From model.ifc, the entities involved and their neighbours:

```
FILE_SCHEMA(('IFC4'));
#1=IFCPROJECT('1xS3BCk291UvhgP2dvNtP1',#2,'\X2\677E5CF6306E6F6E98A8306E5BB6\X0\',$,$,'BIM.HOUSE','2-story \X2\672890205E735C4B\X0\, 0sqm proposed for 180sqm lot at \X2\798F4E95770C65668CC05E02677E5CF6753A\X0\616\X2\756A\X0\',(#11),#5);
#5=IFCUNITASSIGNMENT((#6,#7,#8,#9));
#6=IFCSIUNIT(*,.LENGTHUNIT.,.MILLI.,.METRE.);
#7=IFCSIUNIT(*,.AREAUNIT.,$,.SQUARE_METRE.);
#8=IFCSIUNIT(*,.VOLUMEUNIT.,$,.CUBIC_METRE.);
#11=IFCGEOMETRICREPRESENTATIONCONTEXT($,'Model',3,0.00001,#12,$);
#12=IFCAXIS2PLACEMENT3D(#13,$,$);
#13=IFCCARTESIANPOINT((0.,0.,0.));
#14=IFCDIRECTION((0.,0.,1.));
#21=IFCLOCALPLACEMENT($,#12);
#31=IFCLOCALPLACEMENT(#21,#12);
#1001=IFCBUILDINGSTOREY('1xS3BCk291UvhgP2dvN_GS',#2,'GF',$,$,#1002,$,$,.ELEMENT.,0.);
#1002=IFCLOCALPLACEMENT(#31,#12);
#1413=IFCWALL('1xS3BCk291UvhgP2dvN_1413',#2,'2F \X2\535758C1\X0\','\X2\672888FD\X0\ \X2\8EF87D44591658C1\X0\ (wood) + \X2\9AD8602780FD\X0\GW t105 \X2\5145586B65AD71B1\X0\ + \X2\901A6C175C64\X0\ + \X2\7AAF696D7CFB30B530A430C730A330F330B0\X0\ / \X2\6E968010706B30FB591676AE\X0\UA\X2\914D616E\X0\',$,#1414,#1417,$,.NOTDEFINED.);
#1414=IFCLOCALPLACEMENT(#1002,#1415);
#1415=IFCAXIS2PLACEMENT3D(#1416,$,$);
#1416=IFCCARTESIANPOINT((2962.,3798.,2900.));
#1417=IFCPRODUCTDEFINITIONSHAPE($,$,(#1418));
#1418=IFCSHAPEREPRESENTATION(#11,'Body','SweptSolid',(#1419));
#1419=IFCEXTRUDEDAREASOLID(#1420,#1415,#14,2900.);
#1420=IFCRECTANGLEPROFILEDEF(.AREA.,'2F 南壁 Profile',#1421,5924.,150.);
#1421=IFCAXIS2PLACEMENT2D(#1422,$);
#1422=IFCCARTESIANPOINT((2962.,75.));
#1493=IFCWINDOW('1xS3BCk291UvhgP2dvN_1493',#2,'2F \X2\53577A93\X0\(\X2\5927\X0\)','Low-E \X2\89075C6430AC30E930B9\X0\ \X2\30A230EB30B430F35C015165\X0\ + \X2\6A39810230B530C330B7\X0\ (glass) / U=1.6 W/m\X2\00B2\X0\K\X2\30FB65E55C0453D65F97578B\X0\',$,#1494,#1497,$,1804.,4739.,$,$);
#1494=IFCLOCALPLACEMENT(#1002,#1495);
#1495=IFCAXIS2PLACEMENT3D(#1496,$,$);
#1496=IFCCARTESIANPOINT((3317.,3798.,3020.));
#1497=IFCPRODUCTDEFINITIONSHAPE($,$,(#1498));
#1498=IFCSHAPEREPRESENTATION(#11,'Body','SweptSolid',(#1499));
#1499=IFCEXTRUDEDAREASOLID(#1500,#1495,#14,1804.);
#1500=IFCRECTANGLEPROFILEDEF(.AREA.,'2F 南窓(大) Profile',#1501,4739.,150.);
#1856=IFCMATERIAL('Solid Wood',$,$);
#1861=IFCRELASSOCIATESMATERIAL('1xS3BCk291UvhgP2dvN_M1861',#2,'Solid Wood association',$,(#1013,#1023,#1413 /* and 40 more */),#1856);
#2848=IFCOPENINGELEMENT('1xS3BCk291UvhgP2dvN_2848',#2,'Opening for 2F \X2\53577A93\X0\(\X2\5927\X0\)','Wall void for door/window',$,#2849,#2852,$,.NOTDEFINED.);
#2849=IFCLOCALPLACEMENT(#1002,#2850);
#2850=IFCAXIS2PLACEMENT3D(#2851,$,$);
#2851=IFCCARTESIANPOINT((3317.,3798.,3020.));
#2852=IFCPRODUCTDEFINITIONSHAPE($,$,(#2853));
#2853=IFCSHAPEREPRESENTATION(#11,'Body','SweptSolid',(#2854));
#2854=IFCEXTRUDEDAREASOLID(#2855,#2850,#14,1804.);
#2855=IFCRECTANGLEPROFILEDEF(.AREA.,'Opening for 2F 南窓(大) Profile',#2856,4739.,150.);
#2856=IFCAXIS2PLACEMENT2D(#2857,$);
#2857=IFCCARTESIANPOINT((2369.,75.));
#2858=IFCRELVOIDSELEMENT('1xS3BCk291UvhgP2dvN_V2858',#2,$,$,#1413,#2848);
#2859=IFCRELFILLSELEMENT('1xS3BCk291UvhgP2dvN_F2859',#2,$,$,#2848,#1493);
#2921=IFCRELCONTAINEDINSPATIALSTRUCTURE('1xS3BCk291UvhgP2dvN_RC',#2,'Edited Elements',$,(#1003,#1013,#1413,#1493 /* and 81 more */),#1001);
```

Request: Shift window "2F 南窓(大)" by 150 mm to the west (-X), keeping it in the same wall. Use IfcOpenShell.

```python
import ifcopenshell
import ifcopenshell.api.geometry
import ifcopenshell.util.placement
import ifcopenshell.util.unit

model = ifcopenshell.open("model.ifc")
unit_scale = ifcopenshell.util.unit.calculate_unit_scale(model)

window = model.by_guid("1xS3BCk291UvhgP2dvN_1493")
opening = window.FillsVoids[0].RelatingOpeningElement
wall = opening.VoidsElements[0].RelatingBuildingElement

wall_matrix = ifcopenshell.util.placement.get_local_placement(wall.ObjectPlacement)
shift = wall_matrix[:3, 0] * -0.15 / unit_scale
before = ifcopenshell.util.placement.get_local_placement(window.ObjectPlacement)[:3, 3].copy()

# The window is not placed relative to its opening, so move both.
for product in (opening, window):
    matrix = ifcopenshell.util.placement.get_local_placement(product.ObjectPlacement)
    matrix[:3, 3] += shift
    ifcopenshell.api.geometry.edit_object_placement(model, product=product, matrix=matrix, is_si=False)

after = ifcopenshell.util.placement.get_local_placement(window.ObjectPlacement)[:3, 3]
print("window moved by", (after - before).round(3) + 0.0)

model.write("model-out.ifc")
```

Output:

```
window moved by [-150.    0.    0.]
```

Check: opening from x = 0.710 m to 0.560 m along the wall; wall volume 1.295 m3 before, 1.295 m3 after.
